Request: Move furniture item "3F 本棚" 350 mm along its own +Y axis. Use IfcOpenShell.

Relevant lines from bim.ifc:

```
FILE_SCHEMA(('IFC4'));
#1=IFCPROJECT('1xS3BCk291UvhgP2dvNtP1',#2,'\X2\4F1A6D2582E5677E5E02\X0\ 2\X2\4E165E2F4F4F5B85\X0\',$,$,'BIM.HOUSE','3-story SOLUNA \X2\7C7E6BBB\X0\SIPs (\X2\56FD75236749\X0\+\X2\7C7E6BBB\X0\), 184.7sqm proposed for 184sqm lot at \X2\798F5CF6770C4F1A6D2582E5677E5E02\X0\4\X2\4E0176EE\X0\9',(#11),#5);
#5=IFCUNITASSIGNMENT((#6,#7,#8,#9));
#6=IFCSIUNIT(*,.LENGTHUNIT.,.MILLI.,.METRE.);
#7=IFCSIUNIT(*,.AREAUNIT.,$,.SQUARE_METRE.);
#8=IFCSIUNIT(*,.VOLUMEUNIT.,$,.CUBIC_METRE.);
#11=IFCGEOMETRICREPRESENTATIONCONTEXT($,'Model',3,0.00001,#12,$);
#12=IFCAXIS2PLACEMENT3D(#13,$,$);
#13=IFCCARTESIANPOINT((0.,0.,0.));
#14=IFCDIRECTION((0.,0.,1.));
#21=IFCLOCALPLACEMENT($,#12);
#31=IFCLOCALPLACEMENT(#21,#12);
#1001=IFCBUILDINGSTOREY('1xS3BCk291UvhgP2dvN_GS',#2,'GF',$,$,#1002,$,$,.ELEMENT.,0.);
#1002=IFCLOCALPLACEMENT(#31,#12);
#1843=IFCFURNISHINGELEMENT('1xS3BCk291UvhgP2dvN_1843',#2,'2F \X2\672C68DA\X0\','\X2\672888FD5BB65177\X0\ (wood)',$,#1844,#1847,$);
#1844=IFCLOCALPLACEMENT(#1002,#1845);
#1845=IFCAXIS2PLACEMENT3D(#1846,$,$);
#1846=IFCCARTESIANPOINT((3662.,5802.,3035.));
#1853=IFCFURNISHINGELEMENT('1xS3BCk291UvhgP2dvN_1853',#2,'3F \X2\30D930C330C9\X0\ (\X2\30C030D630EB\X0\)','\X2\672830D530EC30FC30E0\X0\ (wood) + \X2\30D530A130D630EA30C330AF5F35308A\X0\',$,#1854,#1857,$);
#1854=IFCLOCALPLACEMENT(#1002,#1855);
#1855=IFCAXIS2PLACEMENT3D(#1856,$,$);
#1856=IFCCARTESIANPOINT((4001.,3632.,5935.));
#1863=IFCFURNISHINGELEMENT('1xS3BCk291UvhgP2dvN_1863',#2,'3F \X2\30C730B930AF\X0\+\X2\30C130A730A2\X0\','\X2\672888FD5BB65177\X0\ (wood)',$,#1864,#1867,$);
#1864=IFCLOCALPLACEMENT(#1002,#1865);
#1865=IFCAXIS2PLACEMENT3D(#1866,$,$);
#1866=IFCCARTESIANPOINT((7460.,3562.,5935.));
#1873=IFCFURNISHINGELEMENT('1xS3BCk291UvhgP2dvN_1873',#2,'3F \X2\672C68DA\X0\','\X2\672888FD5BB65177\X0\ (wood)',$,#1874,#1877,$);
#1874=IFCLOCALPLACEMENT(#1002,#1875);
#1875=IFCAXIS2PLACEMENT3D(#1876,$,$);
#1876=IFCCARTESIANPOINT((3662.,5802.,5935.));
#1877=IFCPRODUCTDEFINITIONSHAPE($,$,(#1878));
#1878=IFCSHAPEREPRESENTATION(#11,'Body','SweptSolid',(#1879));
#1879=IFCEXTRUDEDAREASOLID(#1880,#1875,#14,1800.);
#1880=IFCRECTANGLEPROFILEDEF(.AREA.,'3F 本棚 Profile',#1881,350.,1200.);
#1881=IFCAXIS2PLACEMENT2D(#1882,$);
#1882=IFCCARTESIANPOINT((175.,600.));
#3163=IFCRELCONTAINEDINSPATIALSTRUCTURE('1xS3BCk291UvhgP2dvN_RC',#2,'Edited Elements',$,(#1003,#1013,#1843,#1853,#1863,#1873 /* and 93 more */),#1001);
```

```python
import ifcopenshell
import ifcopenshell.api.geometry
import ifcopenshell.util.placement
import ifcopenshell.util.unit

model = ifcopenshell.open("bim.ifc")
unit_scale = ifcopenshell.util.unit.calculate_unit_scale(model)

item = model.by_guid("1xS3BCk291UvhgP2dvN_1873")
matrix = ifcopenshell.util.placement.get_local_placement(item.ObjectPlacement)
matrix[:3, 3] += matrix[:3, 1] * 0.35 / unit_scale
ifcopenshell.api.geometry.edit_object_placement(model, product=item, matrix=matrix, is_si=False)

print(ifcopenshell.util.placement.get_local_placement(item.ObjectPlacement).round(3) + 0.0)

model.write("bim_rev.ifc")
```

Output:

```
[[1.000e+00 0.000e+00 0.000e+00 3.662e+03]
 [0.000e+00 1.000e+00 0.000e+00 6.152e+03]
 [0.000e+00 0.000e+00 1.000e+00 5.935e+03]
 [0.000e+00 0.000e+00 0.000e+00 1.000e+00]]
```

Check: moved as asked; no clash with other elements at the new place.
